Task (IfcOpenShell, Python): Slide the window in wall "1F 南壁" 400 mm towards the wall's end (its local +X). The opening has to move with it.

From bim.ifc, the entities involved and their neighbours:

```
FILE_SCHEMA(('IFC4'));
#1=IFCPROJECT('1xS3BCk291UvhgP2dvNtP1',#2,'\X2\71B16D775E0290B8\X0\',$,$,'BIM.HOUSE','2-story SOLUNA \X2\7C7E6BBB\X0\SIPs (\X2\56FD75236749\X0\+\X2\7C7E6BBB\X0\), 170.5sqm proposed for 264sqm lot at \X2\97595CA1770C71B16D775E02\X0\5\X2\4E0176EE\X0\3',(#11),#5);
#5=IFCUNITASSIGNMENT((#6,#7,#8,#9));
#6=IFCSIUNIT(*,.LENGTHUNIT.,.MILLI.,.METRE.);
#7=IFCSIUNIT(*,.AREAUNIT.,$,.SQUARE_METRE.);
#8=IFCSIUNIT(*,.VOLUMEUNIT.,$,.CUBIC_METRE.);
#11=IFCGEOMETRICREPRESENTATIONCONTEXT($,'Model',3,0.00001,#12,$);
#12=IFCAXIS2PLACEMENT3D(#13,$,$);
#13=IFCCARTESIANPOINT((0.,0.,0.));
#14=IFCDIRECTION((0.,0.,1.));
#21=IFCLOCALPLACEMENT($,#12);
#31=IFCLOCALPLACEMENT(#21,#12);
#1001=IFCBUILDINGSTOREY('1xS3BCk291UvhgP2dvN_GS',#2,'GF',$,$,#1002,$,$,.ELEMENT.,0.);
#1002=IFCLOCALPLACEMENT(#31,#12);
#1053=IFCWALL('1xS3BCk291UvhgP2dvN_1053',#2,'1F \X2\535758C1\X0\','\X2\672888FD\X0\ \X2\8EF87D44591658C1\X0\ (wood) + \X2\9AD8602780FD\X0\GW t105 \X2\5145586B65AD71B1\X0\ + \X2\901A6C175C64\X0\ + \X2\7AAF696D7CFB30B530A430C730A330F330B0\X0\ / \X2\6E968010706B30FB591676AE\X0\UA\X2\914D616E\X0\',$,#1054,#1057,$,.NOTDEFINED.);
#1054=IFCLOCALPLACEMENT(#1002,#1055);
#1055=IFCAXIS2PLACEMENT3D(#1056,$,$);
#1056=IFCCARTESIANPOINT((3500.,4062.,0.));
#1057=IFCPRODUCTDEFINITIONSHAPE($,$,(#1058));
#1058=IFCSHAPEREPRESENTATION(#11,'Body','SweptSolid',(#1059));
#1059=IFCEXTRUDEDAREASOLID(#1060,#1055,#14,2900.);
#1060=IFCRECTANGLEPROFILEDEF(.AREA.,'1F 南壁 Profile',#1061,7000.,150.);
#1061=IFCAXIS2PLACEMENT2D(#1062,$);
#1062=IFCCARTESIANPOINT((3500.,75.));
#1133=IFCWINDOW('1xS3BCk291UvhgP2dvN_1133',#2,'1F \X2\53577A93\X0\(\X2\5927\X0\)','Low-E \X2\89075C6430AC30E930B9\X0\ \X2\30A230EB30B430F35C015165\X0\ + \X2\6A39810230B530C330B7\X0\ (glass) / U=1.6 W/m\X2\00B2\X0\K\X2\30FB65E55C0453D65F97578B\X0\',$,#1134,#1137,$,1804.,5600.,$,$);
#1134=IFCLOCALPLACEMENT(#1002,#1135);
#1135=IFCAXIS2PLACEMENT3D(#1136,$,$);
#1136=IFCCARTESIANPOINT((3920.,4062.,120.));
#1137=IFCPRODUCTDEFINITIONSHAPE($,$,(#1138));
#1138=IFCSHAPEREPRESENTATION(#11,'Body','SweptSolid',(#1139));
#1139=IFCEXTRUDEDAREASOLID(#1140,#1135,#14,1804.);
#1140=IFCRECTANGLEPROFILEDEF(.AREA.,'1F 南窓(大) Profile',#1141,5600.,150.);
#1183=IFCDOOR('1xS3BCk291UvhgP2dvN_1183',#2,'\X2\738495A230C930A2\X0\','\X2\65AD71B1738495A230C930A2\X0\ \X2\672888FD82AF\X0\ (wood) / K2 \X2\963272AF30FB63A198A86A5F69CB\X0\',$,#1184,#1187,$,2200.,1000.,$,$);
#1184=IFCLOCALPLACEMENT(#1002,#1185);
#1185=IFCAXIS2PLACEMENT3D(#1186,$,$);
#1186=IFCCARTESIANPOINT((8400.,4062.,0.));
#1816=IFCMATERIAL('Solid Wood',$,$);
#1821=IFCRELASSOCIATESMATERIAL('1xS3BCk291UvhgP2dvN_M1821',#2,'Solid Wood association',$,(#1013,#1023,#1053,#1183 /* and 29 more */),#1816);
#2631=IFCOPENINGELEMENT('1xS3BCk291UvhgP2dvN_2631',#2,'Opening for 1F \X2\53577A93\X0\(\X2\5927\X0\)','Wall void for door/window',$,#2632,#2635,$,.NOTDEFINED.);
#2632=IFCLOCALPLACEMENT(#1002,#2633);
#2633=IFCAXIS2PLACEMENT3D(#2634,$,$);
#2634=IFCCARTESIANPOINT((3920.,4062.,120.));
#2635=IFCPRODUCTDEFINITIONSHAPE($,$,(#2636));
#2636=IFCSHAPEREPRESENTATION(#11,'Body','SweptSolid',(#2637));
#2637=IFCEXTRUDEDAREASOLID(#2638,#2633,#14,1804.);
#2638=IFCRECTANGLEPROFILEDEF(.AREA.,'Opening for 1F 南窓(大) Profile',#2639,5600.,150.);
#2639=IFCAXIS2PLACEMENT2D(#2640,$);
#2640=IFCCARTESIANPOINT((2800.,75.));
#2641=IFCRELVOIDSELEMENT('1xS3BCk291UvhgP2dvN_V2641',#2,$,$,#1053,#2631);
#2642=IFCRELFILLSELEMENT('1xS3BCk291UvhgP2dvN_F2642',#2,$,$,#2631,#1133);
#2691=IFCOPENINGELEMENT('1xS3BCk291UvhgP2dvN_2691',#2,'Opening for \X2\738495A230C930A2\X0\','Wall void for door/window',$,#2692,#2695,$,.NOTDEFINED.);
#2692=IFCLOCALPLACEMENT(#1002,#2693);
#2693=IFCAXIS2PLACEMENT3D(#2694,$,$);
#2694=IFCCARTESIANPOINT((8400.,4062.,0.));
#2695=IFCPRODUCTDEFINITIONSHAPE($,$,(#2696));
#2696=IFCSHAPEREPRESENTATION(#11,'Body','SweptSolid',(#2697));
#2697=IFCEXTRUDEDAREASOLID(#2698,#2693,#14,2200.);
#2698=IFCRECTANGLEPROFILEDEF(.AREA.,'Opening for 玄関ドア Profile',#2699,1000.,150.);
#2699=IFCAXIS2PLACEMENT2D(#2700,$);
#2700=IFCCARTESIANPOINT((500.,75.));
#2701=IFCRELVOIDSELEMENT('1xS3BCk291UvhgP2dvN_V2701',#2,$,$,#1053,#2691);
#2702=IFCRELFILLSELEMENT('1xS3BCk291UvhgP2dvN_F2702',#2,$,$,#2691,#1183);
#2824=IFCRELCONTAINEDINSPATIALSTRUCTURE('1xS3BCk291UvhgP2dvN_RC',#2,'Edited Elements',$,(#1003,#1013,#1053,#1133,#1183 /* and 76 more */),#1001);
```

```python
import ifcopenshell
import ifcopenshell.api.geometry
import ifcopenshell.util.placement
import ifcopenshell.util.unit

model = ifcopenshell.open("bim.ifc")
unit_scale = ifcopenshell.util.unit.calculate_unit_scale(model)

window = model.by_id(1133)
opening = window.FillsVoids[0].RelatingOpeningElement
wall = opening.VoidsElements[0].RelatingBuildingElement

wall_matrix = ifcopenshell.util.placement.get_local_placement(wall.ObjectPlacement)
shift = wall_matrix[:3, 0] * 0.4 / unit_scale
before = ifcopenshell.util.placement.get_local_placement(window.ObjectPlacement)[:3, 3].copy()

# The window is not placed relative to its opening, so move both.
for product in (opening, window):
    matrix = ifcopenshell.util.placement.get_local_placement(product.ObjectPlacement)
    matrix[:3, 3] += shift
    ifcopenshell.api.geometry.edit_object_placement(model, product=product, matrix=matrix, is_si=False)

after = ifcopenshell.util.placement.get_local_placement(window.ObjectPlacement)[:3, 3]
print("window moved by", (after - before).round(3) + 0.0)

model.write("bim_updated.ifc")
```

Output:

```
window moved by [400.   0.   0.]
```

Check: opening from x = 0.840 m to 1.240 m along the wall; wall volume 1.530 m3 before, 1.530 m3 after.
